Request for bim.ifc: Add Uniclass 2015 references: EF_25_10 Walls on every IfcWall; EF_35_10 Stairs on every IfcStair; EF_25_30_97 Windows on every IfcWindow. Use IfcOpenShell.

First a look at what the model holds.

```python
import ifcopenshell

model = ifcopenshell.open("bim.ifc")
print(model.schema)
print("classifications:", [c.Name for c in model.by_type("IfcClassification")])
for ifc_class in ("IfcDoor", "IfcRoof", "IfcStair", "IfcWall", "IfcWindow"):
    print(ifc_class, len(model.by_type(ifc_class)))
```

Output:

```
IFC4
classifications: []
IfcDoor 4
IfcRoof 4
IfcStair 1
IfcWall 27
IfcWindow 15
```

```python
import ifcopenshell
import ifcopenshell.api.classification

model = ifcopenshell.open("bim.ifc")

system = ifcopenshell.api.classification.add_classification(model, classification="Uniclass 2015")

codes = {
    "IfcWall": ("EF_25_10", "Walls"),
    "IfcStair": ("EF_35_10", "Stairs"),
    "IfcWindow": ("EF_25_30_97", "Windows"),
}
for ifc_class, (code, name) in codes.items():
    products = model.by_type(ifc_class)
    ifcopenshell.api.classification.add_reference(
        model, products=products, classification=system, identification=code, name=name
    )
    print(code, len(products))

model.write("bim-out.ifc")
```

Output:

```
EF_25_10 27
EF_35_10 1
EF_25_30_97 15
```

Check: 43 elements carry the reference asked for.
